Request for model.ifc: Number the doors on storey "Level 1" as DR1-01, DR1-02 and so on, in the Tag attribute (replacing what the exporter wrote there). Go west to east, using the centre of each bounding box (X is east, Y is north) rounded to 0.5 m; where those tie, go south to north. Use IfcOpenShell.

First a look at what the model holds.

```python
import ifcopenshell
import ifcopenshell.util.element
import ifcopenshell.util.placement

model = ifcopenshell.open("model.ifc")
print(model.schema)
storey = next(s for s in model.by_type("IfcBuildingStorey") if s.Name == "Level 1")
doors = [e for e in ifcopenshell.util.element.get_decomposition(storey) if e.is_a("IfcDoor")]
for e in sorted(doors, key=lambda e: e.id()):
    origin = ifcopenshell.util.placement.get_local_placement(e.ObjectPlacement)[:3, 3]
    print(e.id(), e.Tag, e.Name, origin.round(2) + 0.0, sep=" | ")
```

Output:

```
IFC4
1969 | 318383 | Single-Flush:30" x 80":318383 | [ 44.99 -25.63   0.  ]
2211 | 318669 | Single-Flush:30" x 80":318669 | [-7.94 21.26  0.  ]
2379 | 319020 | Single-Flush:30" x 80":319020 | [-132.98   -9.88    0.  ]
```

```python
import ifcopenshell
import ifcopenshell.geom
import ifcopenshell.util.element
import ifcopenshell.util.shape

model = ifcopenshell.open("model.ifc")
settings = ifcopenshell.geom.settings()
settings.set("use-world-coords", True)


def centre(element):
    shape = ifcopenshell.geom.create_shape(settings, element)
    return ifcopenshell.util.shape.get_bbox_centroid(shape.geometry)


storey = next(s for s in model.by_type("IfcBuildingStorey") if s.Name == "Level 1")
doors = [e for e in ifcopenshell.util.element.get_decomposition(storey) if e.is_a("IfcDoor")]

# Insertion points can sit at a corner or the storey origin, so sort by the geometry (in metres).
centres = {e: centre(e) for e in doors}
doors.sort(key=lambda e: (round(centres[e][0] / 0.5), centres[e][1]))

for i, e in enumerate(doors, start=1):
    number = f"DR1-{i:02d}"
    e.Tag = number
    print(e.id(), number)

model.write("model_edited.ifc")
```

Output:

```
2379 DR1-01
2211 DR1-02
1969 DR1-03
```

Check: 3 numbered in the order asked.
